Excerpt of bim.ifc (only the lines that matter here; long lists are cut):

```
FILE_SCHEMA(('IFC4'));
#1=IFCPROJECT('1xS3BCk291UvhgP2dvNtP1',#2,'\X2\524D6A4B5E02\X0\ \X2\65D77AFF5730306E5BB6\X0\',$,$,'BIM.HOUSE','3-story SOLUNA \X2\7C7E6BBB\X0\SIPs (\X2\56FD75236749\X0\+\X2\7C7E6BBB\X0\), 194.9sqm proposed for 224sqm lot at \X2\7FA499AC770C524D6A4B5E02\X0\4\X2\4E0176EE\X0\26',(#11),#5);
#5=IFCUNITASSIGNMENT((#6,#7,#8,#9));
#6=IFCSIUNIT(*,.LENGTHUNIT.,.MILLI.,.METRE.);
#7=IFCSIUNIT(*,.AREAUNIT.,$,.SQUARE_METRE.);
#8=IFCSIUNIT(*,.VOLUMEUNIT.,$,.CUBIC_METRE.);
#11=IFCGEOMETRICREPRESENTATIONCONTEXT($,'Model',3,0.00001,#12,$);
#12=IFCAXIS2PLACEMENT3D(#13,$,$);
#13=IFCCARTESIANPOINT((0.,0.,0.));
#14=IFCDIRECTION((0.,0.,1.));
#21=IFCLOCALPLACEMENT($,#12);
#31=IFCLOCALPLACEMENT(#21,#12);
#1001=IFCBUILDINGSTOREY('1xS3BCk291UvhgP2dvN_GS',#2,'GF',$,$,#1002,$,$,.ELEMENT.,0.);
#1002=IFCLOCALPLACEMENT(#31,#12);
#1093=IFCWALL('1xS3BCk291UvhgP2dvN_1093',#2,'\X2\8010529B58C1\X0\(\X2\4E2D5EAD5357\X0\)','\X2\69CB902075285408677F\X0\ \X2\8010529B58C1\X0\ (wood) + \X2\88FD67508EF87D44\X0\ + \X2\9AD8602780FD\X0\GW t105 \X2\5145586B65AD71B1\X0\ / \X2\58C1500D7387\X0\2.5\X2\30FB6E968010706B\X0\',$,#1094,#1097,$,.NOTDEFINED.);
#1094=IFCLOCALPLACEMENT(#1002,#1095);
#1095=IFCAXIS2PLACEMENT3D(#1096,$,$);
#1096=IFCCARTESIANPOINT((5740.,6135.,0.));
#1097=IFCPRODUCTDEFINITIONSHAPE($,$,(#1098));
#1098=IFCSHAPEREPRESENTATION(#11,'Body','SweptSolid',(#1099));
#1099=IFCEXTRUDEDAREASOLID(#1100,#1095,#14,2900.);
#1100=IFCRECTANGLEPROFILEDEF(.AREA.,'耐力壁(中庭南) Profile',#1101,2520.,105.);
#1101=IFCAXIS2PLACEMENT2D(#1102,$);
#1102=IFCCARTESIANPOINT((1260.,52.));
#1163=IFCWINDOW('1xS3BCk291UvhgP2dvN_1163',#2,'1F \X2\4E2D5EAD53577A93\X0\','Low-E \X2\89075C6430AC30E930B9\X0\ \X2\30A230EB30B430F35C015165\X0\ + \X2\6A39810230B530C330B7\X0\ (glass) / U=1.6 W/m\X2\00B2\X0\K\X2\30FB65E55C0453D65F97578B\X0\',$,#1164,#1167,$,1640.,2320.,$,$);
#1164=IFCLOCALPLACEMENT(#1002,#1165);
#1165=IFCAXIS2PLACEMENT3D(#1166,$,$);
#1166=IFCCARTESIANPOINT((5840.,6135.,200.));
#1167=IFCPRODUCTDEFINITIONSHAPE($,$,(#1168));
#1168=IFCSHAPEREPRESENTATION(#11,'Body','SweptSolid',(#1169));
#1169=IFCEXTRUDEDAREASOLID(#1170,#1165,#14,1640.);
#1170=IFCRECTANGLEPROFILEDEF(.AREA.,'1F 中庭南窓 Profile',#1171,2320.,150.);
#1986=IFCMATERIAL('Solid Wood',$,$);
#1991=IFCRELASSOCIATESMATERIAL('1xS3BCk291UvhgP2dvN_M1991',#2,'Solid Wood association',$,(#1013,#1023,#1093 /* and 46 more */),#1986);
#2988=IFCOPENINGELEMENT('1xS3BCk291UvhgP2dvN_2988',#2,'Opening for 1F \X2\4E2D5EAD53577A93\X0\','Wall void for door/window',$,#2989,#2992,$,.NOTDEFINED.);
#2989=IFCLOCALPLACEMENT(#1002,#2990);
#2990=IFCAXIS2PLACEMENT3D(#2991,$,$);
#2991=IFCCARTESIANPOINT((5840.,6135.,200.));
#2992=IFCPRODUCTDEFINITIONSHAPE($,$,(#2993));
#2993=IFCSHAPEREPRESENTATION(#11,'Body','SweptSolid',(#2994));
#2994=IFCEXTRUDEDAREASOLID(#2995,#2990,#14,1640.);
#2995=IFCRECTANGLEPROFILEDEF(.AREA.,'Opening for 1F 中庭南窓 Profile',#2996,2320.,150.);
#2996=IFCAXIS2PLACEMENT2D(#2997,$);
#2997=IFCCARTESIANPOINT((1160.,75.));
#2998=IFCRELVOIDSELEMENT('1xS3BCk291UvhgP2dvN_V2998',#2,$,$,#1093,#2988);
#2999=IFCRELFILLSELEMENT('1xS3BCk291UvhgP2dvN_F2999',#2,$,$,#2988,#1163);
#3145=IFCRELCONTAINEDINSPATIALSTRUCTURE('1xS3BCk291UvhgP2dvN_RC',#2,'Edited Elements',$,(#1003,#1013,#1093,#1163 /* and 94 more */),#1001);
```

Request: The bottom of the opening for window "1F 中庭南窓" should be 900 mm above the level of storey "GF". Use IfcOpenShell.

```python
import numpy as np
import ifcopenshell
import ifcopenshell.api.geometry
import ifcopenshell.geom
import ifcopenshell.util.element
import ifcopenshell.util.placement
import ifcopenshell.util.shape
import ifcopenshell.util.unit

model = ifcopenshell.open("bim.ifc")
unit_scale = ifcopenshell.util.unit.calculate_unit_scale(model)

window = model.by_guid("1xS3BCk291UvhgP2dvN_1163")
opening = window.FillsVoids[0].RelatingOpeningElement
storey = ifcopenshell.util.element.get_container(window, ifc_class="IfcBuildingStorey")
level = ifcopenshell.util.placement.get_local_placement(storey.ObjectPlacement)[2, 3]

# The opening's origin need not be at the sill, so measure its lowest point.
shape = ifcopenshell.geom.create_shape(ifcopenshell.geom.settings(), opening)
bottom = ifcopenshell.util.shape.get_shape_bottom_elevation(shape, shape.geometry) / unit_scale
dz = level + 0.9 / unit_scale - bottom

shift = np.array([0.0, 0.0, dz])
# The window is not placed relative to its opening, so move both.
for product in (opening, window):
    matrix = ifcopenshell.util.placement.get_local_placement(product.ObjectPlacement)
    matrix[:3, 3] += shift
    ifcopenshell.api.geometry.edit_object_placement(model, product=product, matrix=matrix, is_si=False)

print(f"moved by {dz * unit_scale:+.3f} m")

model.write("bim-out.ifc")
```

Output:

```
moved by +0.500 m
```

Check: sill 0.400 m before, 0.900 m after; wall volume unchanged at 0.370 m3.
